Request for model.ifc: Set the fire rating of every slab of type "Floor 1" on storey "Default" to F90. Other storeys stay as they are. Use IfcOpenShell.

First a look at what the model holds.

```python
import ifcopenshell
import ifcopenshell.util.element

model = ifcopenshell.open("model.ifc")
print(model.schema)
storey = next(s for s in model.by_type("IfcBuildingStorey") if s.Name == "Default")
slabs = [e for e in ifcopenshell.util.element.get_decomposition(storey) if e.is_a("IfcSlab")]
seen = {}
for e in slabs:
    element_type = ifcopenshell.util.element.get_type(e)
    key = (element_type.Name if element_type != e and element_type else None, ifcopenshell.util.element.get_pset(e, "Pset_SlabCommon", "FireRating"))
    seen[key] = seen.get(key, 0) + 1
for (name, value), count in sorted(seen.items(), key=str):
    print(count, "x", name, "|", value)
```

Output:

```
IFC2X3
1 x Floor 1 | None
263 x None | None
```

```python
import ifcopenshell
import ifcopenshell.api.pset
import ifcopenshell.util.element

model = ifcopenshell.open("model.ifc")

storey = next(s for s in model.by_type("IfcBuildingStorey") if s.Name == "Default")
slabs = [e for e in ifcopenshell.util.element.get_decomposition(storey) if e.is_a("IfcSlab")]

count = 0
for e in slabs:
    element_type = ifcopenshell.util.element.get_type(e)
    if element_type in (None, e) or element_type.Name != "Floor 1":
        continue
    # add_pset returns the element's existing set when there is one.
    pset = ifcopenshell.api.pset.add_pset(model, product=e, name="Pset_SlabCommon")
    ifcopenshell.api.pset.edit_pset(model, pset=pset, properties={"FireRating": "F90"})
    count += 1

print(count, "slabs updated")

model.write("model_rev.ifc")
```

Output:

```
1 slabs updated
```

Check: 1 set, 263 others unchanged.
